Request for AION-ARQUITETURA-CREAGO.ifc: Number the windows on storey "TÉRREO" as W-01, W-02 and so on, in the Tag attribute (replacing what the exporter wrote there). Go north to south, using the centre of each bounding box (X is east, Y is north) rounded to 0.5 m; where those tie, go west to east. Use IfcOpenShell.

First a look at what the model holds.

```python
import ifcopenshell
import ifcopenshell.util.element
import ifcopenshell.util.placement

model = ifcopenshell.open("AION-ARQUITETURA-CREAGO.ifc")
print(model.schema)
storey = next(s for s in model.by_type("IfcBuildingStorey") if s.Name == "TÉRREO")
windows = [e for e in ifcopenshell.util.element.get_decomposition(storey) if e.is_a("IfcWindow")]
for e in sorted(windows, key=lambda e: e.id()):
    origin = ifcopenshell.util.placement.get_local_placement(e.ObjectPlacement)[:3, 3]
    print(e.id(), e.Tag, e.Name, origin.round(2) + 0.0, sep=" | ")
```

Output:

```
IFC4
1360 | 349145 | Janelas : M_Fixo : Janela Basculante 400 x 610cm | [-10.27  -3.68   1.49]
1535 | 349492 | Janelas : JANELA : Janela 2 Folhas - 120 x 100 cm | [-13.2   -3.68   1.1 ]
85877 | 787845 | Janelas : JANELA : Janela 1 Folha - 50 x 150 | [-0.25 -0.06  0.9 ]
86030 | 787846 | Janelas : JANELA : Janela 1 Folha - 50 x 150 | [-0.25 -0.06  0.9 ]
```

```python
import ifcopenshell
import ifcopenshell.geom
import ifcopenshell.util.element
import ifcopenshell.util.shape

model = ifcopenshell.open("AION-ARQUITETURA-CREAGO.ifc")
settings = ifcopenshell.geom.settings()
settings.set("use-world-coords", True)


def centre(element):
    shape = ifcopenshell.geom.create_shape(settings, element)
    return ifcopenshell.util.shape.get_bbox_centroid(shape.geometry)


storey = next(s for s in model.by_type("IfcBuildingStorey") if s.Name == "TÉRREO")
windows = [e for e in ifcopenshell.util.element.get_decomposition(storey) if e.is_a("IfcWindow")]

# Insertion points can sit at a corner or the storey origin, so sort by the geometry (in metres).
centres = {e: centre(e) for e in windows}
windows.sort(key=lambda e: (-round(centres[e][1] / 0.5), centres[e][0]))

for i, e in enumerate(windows, start=1):
    number = f"W-{i:02d}"
    e.Tag = number
    print(e.id(), number)

model.write("AION-ARQUITETURA-CREAGO_updated.ifc")
```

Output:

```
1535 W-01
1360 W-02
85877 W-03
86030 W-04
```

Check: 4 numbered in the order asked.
